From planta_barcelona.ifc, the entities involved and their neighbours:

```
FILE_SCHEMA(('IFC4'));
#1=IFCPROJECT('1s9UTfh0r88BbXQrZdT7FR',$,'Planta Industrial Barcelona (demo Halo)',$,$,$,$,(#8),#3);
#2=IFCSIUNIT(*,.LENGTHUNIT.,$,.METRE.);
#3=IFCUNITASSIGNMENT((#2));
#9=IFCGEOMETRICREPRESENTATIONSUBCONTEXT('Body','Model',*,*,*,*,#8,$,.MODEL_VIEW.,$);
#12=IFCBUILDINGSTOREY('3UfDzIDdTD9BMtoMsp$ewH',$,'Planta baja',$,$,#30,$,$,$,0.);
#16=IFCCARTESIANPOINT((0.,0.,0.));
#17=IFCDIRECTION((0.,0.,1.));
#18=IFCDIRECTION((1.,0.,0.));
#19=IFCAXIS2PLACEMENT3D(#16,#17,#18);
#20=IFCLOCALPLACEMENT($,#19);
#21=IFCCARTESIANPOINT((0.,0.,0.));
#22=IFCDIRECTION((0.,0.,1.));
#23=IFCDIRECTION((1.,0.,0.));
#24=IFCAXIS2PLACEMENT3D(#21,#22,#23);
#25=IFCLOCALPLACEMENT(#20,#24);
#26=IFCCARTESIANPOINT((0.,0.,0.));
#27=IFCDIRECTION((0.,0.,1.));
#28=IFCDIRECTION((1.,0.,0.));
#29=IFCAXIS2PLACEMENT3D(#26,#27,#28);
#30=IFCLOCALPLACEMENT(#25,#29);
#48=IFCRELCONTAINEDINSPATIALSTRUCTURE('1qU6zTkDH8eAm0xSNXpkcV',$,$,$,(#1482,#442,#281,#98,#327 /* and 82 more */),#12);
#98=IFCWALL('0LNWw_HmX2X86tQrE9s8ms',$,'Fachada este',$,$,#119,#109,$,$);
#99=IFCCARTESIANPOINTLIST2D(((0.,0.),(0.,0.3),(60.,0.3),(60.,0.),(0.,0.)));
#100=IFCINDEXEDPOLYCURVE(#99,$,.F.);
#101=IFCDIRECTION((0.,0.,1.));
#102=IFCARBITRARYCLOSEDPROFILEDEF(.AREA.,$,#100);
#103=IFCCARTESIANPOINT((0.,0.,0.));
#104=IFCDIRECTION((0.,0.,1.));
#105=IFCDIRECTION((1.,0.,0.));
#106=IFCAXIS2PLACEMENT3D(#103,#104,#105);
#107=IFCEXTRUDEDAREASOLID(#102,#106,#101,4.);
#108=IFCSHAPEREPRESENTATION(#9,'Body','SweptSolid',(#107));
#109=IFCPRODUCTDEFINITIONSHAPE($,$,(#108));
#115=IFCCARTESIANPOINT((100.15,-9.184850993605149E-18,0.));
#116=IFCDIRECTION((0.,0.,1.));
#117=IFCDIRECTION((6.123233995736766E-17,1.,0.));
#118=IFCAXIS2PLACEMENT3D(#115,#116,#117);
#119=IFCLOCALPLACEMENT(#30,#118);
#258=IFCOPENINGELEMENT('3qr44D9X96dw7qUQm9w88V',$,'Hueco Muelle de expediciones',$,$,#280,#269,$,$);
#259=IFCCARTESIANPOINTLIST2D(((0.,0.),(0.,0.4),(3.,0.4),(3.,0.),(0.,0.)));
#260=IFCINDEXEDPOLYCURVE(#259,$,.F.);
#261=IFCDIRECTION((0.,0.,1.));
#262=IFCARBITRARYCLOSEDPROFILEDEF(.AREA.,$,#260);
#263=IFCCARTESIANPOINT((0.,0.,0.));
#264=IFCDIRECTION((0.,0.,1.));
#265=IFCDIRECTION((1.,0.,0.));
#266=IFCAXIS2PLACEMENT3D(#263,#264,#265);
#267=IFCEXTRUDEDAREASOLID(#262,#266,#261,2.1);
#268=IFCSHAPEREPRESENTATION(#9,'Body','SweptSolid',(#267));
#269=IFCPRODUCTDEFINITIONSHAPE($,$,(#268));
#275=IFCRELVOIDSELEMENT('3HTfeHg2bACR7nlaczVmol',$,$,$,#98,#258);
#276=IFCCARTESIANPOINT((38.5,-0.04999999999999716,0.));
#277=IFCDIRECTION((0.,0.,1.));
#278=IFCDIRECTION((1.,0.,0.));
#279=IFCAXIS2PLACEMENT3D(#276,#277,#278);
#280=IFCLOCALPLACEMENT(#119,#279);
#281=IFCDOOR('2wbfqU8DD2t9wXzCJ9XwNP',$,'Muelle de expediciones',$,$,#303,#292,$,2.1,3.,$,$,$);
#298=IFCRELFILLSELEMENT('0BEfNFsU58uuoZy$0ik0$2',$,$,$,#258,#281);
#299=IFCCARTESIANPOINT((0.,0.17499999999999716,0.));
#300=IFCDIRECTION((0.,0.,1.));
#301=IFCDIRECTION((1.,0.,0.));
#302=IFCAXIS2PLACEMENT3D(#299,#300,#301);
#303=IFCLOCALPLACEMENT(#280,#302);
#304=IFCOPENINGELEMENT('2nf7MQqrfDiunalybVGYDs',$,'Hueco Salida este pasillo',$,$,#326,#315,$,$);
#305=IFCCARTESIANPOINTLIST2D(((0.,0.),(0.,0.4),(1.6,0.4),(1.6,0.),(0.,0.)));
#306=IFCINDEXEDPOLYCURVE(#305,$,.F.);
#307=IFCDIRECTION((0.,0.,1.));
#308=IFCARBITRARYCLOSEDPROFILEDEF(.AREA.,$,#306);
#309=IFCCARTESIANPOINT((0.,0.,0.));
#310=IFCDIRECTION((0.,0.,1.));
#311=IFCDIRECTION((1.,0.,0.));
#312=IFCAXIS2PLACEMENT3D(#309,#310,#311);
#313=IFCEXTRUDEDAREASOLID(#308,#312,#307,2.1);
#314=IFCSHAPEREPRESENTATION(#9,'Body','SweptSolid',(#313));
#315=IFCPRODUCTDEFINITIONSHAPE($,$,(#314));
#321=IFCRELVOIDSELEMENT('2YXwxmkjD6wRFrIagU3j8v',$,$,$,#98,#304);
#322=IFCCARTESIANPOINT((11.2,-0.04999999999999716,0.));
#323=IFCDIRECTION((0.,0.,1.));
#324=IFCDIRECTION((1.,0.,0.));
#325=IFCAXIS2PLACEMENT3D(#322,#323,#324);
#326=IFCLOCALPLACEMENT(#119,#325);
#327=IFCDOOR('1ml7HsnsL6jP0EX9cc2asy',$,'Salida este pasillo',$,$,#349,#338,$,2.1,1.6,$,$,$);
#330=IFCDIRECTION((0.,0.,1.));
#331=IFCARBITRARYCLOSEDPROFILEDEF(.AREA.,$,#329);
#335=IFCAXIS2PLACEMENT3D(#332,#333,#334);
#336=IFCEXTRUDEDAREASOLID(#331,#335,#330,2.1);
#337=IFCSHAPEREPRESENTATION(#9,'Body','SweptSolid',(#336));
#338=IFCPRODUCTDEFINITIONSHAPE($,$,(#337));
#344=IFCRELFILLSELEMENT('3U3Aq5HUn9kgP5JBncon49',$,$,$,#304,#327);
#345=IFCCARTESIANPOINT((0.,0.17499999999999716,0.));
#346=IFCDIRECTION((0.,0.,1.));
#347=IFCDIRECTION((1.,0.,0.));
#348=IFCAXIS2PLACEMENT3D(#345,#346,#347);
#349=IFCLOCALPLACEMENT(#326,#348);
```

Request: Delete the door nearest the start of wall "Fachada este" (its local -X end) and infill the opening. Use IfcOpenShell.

```python
import ifcopenshell
import ifcopenshell.api.feature
import ifcopenshell.api.root
import ifcopenshell.geom
import ifcopenshell.util.shape

model = ifcopenshell.open("planta_barcelona.ifc")
settings = ifcopenshell.geom.settings()


def volume(element):
    """Net volume in cubic metres, openings subtracted."""
    shape = ifcopenshell.geom.create_shape(settings, element)
    return ifcopenshell.util.shape.get_volume(shape.geometry)


door = model.by_guid("1ml7HsnsL6jP0EX9cc2asy")
opening = door.FillsVoids[0].RelatingOpeningElement
wall = opening.VoidsElements[0].RelatingBuildingElement
before = volume(wall)

ifcopenshell.api.root.remove_product(model, product=door)
ifcopenshell.api.feature.remove_feature(model, feature=opening)

after = volume(wall)

print(f"wall volume {before:.3f} -> {after:.3f} m3")

model.write("planta_barcelona_rev.ifc")
```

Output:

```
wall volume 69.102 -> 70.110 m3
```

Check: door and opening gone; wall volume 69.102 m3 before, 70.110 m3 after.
